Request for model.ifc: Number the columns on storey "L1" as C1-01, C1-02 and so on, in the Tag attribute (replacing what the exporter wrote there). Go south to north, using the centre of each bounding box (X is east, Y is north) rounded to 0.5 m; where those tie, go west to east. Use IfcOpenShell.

First a look at what the model holds.

```python
import ifcopenshell
import ifcopenshell.util.element
import ifcopenshell.util.placement

model = ifcopenshell.open("model.ifc")
print(model.schema)
storey = next(s for s in model.by_type("IfcBuildingStorey") if s.Name == "L1")
columns = [e for e in ifcopenshell.util.element.get_decomposition(storey) if e.is_a("IfcColumn")]
for e in sorted(columns, key=lambda e: e.id()):
    origin = ifcopenshell.util.placement.get_local_placement(e.ObjectPlacement)[:3, 3]
    print(e.id(), e.Tag, e.Name, origin.round(2) + 0.0, sep=" | ")
```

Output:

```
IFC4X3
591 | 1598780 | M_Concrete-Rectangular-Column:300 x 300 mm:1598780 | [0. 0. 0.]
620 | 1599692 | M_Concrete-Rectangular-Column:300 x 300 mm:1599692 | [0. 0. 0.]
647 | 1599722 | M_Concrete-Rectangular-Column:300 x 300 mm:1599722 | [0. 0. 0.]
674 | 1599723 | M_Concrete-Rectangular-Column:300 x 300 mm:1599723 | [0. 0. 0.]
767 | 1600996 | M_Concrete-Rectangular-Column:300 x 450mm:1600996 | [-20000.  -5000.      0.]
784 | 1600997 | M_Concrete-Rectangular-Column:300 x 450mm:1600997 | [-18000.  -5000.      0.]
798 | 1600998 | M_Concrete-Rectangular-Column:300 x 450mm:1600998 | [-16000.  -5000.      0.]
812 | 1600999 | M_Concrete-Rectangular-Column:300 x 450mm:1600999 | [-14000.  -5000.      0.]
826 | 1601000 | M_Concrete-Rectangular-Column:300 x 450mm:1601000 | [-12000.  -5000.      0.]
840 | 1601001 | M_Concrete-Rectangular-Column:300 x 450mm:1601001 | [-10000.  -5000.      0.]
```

```python
import ifcopenshell
import ifcopenshell.geom
import ifcopenshell.util.element
import ifcopenshell.util.shape

model = ifcopenshell.open("model.ifc")
settings = ifcopenshell.geom.settings()
settings.set("use-world-coords", True)


def centre(element):
    shape = ifcopenshell.geom.create_shape(settings, element)
    return ifcopenshell.util.shape.get_bbox_centroid(shape.geometry)


storey = next(s for s in model.by_type("IfcBuildingStorey") if s.Name == "L1")
columns = [e for e in ifcopenshell.util.element.get_decomposition(storey) if e.is_a("IfcColumn")]

# Insertion points can sit at a corner or the storey origin, so sort by the geometry (in metres).
centres = {e: centre(e) for e in columns}
columns.sort(key=lambda e: (round(centres[e][1] / 0.5), centres[e][0]))

for i, e in enumerate(columns, start=1):
    number = f"C1-{i:02d}"
    e.Tag = number
    print(e.id(), number)

model.write("model_updated.ifc")
```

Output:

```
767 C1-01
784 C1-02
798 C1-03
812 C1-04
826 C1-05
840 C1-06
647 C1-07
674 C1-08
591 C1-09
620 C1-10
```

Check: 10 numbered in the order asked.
